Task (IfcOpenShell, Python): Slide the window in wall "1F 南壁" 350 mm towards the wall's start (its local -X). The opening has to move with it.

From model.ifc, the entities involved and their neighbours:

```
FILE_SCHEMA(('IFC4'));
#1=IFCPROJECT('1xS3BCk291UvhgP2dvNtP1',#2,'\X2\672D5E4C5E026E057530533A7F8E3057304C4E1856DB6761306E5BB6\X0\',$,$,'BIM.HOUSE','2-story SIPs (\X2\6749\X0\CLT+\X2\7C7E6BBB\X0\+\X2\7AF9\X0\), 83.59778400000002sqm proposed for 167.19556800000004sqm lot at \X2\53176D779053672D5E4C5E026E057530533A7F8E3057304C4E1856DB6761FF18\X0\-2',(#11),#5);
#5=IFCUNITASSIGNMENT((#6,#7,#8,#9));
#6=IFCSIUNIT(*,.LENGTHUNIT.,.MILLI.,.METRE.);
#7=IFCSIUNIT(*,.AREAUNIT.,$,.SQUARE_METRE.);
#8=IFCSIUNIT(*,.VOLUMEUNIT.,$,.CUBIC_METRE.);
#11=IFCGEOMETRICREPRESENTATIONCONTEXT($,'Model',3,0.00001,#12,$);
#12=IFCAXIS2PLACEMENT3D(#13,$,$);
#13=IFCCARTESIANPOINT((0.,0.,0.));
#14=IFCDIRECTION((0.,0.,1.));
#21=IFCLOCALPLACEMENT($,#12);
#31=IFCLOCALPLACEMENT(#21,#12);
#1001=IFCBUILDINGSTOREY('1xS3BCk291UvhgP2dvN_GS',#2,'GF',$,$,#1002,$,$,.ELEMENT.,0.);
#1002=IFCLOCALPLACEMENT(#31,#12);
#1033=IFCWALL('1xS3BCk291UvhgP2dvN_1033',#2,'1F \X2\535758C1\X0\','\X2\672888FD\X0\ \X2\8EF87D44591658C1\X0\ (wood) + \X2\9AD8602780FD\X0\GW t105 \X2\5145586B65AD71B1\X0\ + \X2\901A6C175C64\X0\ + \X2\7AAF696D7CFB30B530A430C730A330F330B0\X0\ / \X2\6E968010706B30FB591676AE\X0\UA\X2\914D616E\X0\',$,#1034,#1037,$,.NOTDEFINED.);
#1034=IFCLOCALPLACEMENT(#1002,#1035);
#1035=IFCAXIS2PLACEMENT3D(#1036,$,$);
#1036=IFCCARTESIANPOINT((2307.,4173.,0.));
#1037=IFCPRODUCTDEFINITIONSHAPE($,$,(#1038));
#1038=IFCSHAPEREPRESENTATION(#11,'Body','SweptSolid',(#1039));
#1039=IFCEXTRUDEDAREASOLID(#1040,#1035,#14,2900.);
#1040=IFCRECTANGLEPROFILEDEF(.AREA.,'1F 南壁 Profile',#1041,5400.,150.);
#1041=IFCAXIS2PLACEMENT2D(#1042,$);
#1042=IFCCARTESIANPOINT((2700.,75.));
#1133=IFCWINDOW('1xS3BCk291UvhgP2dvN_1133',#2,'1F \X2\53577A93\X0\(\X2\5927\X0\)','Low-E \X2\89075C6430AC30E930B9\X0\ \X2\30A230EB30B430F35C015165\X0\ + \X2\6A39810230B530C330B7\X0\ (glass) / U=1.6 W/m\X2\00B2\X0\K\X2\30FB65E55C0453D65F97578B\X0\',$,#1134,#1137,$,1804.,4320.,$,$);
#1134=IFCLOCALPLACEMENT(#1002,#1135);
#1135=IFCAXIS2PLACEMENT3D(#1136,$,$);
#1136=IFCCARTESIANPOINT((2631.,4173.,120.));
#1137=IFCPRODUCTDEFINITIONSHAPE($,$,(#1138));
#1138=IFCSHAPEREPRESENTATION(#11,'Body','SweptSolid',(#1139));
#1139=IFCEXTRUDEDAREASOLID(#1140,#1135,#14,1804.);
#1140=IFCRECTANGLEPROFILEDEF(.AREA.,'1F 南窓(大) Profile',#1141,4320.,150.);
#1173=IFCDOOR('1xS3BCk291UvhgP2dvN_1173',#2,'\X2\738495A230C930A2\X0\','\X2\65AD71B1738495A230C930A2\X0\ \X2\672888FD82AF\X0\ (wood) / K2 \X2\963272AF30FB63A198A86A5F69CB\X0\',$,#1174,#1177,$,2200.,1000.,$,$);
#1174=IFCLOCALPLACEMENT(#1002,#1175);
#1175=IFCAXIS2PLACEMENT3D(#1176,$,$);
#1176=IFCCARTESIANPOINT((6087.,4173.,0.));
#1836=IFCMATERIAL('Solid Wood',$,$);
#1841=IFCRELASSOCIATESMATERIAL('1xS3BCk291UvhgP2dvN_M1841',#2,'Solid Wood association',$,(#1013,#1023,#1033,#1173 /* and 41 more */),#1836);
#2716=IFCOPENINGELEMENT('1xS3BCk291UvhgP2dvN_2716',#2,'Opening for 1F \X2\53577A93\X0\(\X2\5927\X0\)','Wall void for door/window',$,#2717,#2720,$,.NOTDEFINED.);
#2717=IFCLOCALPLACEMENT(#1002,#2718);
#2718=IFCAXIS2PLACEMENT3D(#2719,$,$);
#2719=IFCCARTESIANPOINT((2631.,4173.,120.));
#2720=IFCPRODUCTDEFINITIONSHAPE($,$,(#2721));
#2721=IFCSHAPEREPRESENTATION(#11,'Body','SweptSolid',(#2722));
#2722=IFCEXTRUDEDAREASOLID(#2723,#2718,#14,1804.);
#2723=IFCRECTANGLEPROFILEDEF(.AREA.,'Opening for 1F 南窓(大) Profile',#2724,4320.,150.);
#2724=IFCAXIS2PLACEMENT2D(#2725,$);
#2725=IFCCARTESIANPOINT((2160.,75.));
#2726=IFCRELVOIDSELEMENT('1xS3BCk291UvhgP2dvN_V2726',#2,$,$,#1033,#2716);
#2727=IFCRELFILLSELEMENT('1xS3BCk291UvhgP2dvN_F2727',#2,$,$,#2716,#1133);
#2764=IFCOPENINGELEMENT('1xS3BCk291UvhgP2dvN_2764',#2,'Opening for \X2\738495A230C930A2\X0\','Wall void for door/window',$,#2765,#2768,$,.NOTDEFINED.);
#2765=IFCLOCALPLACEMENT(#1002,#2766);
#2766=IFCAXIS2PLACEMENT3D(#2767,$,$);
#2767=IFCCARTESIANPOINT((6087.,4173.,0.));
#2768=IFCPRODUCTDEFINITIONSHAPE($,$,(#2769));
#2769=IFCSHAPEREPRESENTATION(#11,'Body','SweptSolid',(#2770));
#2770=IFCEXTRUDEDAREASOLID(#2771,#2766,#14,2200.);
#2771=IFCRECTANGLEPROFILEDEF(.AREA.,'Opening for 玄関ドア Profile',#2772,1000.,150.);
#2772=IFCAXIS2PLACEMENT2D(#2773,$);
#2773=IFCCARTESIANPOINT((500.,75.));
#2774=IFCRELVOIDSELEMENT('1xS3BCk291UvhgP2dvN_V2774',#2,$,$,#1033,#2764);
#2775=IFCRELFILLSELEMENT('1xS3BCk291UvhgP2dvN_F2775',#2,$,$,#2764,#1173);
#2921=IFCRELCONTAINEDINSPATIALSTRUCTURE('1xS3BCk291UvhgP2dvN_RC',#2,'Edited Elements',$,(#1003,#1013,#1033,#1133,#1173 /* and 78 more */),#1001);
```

```python
import ifcopenshell
import ifcopenshell.api.geometry
import ifcopenshell.util.placement
import ifcopenshell.util.unit

model = ifcopenshell.open("model.ifc")
unit_scale = ifcopenshell.util.unit.calculate_unit_scale(model)

window = model.by_guid("1xS3BCk291UvhgP2dvN_1133")
opening = window.FillsVoids[0].RelatingOpeningElement
wall = opening.VoidsElements[0].RelatingBuildingElement

wall_matrix = ifcopenshell.util.placement.get_local_placement(wall.ObjectPlacement)
shift = wall_matrix[:3, 0] * -0.35 / unit_scale
before = ifcopenshell.util.placement.get_local_placement(window.ObjectPlacement)[:3, 3].copy()

# The window is not placed relative to its opening, so move both.
for product in (opening, window):
    matrix = ifcopenshell.util.placement.get_local_placement(product.ObjectPlacement)
    matrix[:3, 3] += shift
    ifcopenshell.api.geometry.edit_object_placement(model, product=product, matrix=matrix, is_si=False)

after = ifcopenshell.util.placement.get_local_placement(window.ObjectPlacement)[:3, 3]
print("window moved by", (after - before).round(3) + 0.0)

model.write("model_edited.ifc")
```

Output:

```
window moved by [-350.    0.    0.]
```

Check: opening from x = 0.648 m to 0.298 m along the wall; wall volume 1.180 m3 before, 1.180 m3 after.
